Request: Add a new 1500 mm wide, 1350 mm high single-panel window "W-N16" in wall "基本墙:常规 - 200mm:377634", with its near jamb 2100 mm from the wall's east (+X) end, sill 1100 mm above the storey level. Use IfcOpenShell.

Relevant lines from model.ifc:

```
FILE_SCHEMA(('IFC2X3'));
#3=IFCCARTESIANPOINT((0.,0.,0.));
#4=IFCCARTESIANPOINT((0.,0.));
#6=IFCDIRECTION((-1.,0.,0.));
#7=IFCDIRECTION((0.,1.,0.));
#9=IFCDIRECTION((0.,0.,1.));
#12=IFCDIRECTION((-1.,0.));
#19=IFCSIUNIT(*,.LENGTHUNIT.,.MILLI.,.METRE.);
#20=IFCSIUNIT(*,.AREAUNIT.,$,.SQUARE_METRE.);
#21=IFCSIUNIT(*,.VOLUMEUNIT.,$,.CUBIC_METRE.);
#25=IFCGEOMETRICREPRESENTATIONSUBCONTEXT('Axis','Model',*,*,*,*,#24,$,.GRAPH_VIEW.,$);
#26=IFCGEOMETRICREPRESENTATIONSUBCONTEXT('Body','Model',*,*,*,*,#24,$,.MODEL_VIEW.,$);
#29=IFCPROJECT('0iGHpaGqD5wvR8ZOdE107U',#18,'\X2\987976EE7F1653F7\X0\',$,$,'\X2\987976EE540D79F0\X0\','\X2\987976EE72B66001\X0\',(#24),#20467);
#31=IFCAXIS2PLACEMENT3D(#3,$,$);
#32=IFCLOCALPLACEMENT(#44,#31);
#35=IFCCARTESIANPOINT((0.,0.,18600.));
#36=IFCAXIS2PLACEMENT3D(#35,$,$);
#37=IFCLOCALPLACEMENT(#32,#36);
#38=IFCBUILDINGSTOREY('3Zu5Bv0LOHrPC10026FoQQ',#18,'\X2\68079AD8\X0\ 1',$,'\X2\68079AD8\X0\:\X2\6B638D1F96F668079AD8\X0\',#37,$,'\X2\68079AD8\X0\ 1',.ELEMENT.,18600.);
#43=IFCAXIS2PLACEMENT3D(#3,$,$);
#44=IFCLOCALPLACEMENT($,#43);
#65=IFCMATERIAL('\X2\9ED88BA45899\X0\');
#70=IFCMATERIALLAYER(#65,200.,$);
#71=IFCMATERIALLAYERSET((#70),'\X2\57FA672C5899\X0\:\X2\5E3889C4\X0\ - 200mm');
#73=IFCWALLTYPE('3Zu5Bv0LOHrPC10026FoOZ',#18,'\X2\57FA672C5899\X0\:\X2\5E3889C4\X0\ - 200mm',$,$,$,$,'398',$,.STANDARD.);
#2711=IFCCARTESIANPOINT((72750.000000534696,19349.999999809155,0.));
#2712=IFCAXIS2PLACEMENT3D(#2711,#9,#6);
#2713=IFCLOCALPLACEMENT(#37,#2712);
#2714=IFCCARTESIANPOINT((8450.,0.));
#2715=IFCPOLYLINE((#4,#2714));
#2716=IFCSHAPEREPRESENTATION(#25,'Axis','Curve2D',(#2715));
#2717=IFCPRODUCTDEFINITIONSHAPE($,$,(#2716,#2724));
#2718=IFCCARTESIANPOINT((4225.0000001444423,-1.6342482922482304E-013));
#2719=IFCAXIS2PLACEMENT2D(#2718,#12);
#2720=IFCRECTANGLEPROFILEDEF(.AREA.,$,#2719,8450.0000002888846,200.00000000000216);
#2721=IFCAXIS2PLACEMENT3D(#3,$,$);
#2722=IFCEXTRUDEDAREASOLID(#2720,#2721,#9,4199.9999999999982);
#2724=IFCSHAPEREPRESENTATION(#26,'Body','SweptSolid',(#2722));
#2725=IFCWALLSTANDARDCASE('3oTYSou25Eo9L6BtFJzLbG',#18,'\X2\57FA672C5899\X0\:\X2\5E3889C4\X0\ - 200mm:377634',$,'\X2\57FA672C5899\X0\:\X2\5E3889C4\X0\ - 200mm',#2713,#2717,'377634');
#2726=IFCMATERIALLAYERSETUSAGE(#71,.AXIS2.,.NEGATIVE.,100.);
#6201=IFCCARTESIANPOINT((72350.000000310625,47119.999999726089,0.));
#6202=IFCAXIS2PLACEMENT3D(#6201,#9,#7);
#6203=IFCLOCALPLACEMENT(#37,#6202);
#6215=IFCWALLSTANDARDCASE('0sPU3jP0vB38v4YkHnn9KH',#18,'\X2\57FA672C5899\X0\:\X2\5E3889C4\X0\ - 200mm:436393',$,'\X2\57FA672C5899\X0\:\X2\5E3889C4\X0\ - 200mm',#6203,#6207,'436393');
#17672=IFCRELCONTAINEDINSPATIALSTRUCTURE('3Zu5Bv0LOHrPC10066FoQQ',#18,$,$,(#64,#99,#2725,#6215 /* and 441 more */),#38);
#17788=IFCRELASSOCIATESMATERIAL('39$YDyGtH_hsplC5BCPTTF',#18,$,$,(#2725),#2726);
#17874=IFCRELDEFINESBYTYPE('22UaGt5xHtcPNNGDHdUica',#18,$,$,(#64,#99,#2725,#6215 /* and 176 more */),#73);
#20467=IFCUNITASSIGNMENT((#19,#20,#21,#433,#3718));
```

```python
import numpy as np
import ifcopenshell
import ifcopenshell.api.feature
import ifcopenshell.api.geometry
import ifcopenshell.api.root
import ifcopenshell.api.spatial
import ifcopenshell.api.type
import ifcopenshell.geom
import ifcopenshell.util.element
import ifcopenshell.util.placement
import ifcopenshell.util.representation
import ifcopenshell.util.shape
import ifcopenshell.util.unit

model = ifcopenshell.open("model.ifc")
unit_scale = ifcopenshell.util.unit.calculate_unit_scale(model)
settings = ifcopenshell.geom.settings()


def volume(element):
    """Net volume in cubic metres, openings subtracted."""
    shape = ifcopenshell.geom.create_shape(settings, element)
    return ifcopenshell.util.shape.get_volume(shape.geometry)


wall = model.by_guid("3oTYSou25Eo9L6BtFJzLbG")
storey = ifcopenshell.util.element.get_container(wall, ifc_class="IfcBuildingStorey")
context = ifcopenshell.util.representation.get_context(model, "Model", "Body", "MODEL_VIEW")
before = volume(wall)

width, height, from_end, sill = 1.5, 1.35, 2.1, 1.1  # metres

# The wall runs along its own X axis, and the end named is its -X end.
wall_shape = ifcopenshell.geom.create_shape(settings, wall)
x, y, z = ifcopenshell.util.shape.get_vertices(wall_shape.geometry).T
start = x.min() + from_end
face, thickness = float(y.min()), float(y.max() - y.min())
wall_matrix = ifcopenshell.util.placement.get_local_placement(wall.ObjectPlacement)
level = ifcopenshell.util.placement.get_local_placement(storey.ObjectPlacement)[2, 3]


def in_wall(x, y):
    """Placement at x, y metres in the wall's axes, at sill height."""
    matrix = wall_matrix.copy()
    matrix[:, 3] = wall_matrix @ np.array([x / unit_scale, y / unit_scale, 0.0, 1.0])
    matrix[2, 3] = level + sill / unit_scale
    return matrix


# Opening: a box that overshoots both wall faces by 50 mm.
opening = ifcopenshell.api.root.create_entity(model, ifc_class="IfcOpeningElement")
box = ifcopenshell.api.geometry.add_wall_representation(
    model, context=context, length=width, height=height, thickness=thickness + 0.1
)
ifcopenshell.api.geometry.assign_representation(model, product=opening, representation=box)
ifcopenshell.api.geometry.edit_object_placement(model, product=opening, matrix=in_wall(start, face - 0.05), is_si=False)
ifcopenshell.api.feature.add_feature(model, feature=opening, element=wall)

window = ifcopenshell.api.root.create_entity(model, ifc_class="IfcWindow", name="W-N16")
window.OverallWidth, window.OverallHeight = width / unit_scale, height / unit_scale
body = ifcopenshell.api.geometry.add_window_representation(
    model,
    context=context,
    overall_width=window.OverallWidth,
    overall_height=window.OverallHeight,
    partition_type="SINGLE_PANEL",
)
ifcopenshell.api.geometry.assign_representation(model, product=window, representation=body)
ifcopenshell.api.spatial.assign_container(model, products=[window], relating_structure=storey)
fills = ifcopenshell.api.feature.add_filling(model, opening=opening, element=window)
fills.OwnerHistory = window.OwnerHistory  # required in IFC2X3

# IFC2X3 keeps the operation on the window style.
style = ifcopenshell.api.root.create_entity(model, ifc_class="IfcWindowStyle", name="W-N16")
style.OperationType, style.ConstructionType = "SINGLE_PANEL", "NOTDEFINED"
style.ParameterTakesPrecedence = style.Sizeable = False
ifcopenshell.api.type.assign_type(model, related_objects=[window], relating_type=style)

# Centre the window in the wall's thickness.
ifcopenshell.api.geometry.edit_object_placement(model, product=window, matrix=in_wall(start, face), is_si=False)
window_shape = ifcopenshell.geom.create_shape(settings, window)
depth = ifcopenshell.util.shape.get_vertices(window_shape.geometry)[:, 1]
offset = face + thickness / 2 - (depth.min() + depth.max()) / 2
ifcopenshell.api.geometry.edit_object_placement(model, product=window, matrix=in_wall(start, offset), is_si=False)

after = volume(wall)

print(f"wall volume {before:.3f} -> {after:.3f} m3")

model.write("model_edited.ifc")
```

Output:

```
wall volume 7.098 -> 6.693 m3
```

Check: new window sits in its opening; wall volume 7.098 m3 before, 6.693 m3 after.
